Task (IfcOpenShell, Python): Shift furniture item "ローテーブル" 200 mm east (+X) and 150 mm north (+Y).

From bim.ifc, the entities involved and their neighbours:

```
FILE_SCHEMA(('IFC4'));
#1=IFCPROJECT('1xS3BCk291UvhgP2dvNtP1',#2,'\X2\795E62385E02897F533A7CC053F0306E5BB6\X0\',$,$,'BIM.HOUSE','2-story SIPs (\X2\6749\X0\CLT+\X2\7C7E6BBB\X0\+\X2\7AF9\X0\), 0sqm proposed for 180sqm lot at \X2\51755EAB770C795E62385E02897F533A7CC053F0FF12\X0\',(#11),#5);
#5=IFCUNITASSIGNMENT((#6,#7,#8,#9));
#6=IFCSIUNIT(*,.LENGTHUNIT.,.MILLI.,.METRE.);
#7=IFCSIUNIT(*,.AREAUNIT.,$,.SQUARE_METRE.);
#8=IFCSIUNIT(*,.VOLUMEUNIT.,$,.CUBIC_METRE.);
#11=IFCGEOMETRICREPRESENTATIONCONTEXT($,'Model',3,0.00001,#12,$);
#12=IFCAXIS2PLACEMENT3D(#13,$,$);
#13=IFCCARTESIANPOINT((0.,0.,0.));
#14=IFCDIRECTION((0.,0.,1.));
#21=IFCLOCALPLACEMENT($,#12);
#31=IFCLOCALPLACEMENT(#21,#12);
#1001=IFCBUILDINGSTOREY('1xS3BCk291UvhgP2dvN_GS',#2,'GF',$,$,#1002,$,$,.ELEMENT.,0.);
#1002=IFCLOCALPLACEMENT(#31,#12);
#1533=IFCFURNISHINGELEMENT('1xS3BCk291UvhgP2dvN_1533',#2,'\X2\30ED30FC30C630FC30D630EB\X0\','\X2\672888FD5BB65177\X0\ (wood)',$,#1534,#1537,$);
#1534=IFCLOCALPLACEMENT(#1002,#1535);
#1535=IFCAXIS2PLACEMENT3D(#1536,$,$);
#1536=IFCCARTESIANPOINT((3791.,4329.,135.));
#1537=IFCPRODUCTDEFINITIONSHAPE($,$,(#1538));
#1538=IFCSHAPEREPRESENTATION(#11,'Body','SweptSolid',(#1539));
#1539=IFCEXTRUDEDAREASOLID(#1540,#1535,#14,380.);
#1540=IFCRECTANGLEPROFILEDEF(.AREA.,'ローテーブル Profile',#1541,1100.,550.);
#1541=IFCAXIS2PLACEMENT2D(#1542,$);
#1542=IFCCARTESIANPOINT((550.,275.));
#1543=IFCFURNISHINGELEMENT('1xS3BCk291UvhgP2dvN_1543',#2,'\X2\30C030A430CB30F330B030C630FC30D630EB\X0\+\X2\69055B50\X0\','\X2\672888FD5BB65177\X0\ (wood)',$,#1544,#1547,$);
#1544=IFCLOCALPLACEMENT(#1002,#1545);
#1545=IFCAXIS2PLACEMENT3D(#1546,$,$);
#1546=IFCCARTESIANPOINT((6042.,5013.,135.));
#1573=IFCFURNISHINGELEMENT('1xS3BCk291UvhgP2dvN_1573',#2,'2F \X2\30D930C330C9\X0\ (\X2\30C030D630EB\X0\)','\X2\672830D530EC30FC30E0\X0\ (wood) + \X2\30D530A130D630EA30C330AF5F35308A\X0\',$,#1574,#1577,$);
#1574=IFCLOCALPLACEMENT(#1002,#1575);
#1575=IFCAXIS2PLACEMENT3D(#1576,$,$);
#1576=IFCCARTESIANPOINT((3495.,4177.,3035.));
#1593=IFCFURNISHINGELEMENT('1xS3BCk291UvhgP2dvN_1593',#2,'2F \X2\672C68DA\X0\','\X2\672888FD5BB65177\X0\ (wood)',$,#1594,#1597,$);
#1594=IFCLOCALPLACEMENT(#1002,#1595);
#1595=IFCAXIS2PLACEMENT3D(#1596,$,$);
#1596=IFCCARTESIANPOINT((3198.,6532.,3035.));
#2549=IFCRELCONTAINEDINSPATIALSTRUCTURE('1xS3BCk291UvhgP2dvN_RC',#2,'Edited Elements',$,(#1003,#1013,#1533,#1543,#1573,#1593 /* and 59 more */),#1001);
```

```python
import ifcopenshell
import ifcopenshell.api.geometry
import ifcopenshell.util.placement

model = ifcopenshell.open("bim.ifc")

item = model.by_guid("1xS3BCk291UvhgP2dvN_1533")
matrix = ifcopenshell.util.placement.get_local_placement(item.ObjectPlacement)
matrix[0, 3] += 200.0
matrix[1, 3] += 150.0
ifcopenshell.api.geometry.edit_object_placement(model, product=item, matrix=matrix, is_si=False)

print(ifcopenshell.util.placement.get_local_placement(item.ObjectPlacement).round(3) + 0.0)

model.write("bim_rev.ifc")
```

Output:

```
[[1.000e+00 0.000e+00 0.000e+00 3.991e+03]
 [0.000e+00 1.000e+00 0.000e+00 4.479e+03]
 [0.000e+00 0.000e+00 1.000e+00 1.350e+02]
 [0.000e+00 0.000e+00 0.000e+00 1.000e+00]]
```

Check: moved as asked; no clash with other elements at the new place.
